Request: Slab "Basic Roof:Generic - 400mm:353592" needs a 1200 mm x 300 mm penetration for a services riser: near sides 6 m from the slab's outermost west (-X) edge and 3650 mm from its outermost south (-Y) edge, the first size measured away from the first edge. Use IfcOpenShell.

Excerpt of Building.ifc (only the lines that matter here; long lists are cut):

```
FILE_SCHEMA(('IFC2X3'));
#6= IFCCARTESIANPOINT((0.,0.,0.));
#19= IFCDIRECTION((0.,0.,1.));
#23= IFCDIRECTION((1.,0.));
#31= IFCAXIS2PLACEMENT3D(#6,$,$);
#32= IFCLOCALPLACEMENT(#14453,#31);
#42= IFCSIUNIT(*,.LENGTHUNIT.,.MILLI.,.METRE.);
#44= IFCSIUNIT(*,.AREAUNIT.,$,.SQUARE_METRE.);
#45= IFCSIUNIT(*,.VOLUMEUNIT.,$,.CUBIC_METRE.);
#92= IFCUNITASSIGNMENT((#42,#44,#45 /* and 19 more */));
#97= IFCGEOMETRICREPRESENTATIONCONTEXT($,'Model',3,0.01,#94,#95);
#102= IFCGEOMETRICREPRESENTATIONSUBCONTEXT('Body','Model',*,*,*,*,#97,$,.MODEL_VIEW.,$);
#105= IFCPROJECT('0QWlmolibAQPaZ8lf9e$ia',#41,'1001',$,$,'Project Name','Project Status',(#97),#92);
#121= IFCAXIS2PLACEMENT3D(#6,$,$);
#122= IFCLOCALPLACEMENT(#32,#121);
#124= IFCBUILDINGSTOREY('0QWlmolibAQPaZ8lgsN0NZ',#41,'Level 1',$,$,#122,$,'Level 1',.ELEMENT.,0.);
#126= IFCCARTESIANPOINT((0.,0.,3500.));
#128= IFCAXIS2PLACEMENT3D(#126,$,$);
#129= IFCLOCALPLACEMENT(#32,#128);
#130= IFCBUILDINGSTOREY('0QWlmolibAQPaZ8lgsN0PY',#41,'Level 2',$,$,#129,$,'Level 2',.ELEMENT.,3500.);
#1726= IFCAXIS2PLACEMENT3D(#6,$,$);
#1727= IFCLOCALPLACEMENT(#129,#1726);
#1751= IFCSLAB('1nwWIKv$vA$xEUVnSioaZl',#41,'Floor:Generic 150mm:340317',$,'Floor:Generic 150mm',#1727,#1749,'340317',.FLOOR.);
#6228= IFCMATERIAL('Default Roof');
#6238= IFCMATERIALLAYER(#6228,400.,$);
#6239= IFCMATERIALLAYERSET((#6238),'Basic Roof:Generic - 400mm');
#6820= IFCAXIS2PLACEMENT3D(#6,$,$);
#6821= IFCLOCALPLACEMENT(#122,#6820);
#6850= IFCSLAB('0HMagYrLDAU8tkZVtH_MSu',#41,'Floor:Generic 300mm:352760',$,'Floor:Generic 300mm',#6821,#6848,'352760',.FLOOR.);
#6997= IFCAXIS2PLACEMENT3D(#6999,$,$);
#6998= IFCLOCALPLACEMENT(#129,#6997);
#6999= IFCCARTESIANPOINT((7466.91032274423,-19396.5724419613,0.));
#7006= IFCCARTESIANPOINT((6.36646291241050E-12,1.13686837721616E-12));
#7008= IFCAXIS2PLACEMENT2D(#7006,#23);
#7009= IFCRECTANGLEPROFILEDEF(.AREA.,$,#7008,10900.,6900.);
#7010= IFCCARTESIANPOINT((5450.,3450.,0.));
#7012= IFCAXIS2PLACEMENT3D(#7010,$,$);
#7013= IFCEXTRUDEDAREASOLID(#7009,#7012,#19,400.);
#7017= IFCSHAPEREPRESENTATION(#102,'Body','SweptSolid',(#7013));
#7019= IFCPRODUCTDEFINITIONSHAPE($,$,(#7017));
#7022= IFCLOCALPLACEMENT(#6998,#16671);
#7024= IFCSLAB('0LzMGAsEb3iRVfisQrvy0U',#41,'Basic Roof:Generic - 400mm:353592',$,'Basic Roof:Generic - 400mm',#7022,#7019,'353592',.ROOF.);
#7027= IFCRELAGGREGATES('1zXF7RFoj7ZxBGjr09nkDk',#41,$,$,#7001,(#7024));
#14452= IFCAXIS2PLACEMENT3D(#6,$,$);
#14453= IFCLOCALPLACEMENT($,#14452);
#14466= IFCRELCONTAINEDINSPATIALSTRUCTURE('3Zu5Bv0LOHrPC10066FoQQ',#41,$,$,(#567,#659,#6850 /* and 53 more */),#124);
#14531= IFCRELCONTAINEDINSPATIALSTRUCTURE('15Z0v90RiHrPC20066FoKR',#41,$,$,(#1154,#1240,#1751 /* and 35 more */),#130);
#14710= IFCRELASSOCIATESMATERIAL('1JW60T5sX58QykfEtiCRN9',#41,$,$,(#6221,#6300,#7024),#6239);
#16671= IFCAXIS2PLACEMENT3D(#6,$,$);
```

```python
import numpy as np
import ifcopenshell
import ifcopenshell.api.feature
import ifcopenshell.api.geometry
import ifcopenshell.api.root
import ifcopenshell.geom
import ifcopenshell.util.placement
import ifcopenshell.util.representation
import ifcopenshell.util.shape
import ifcopenshell.util.unit

model = ifcopenshell.open("Building.ifc")
unit_scale = ifcopenshell.util.unit.calculate_unit_scale(model)
settings = ifcopenshell.geom.settings()


def volume(element):
    """Net volume in cubic metres, openings subtracted."""
    shape = ifcopenshell.geom.create_shape(settings, element)
    return ifcopenshell.util.shape.get_volume(shape.geometry)


slab = model.by_guid("0LzMGAsEb3iRVfisQrvy0U")
before = volume(slab)

# Extent in the slab's own axes, in metres. The edges named are its -X and -Y sides.
slab_shape = ifcopenshell.geom.create_shape(settings, slab)
vertices = ifcopenshell.util.shape.get_vertices(slab_shape.geometry)
x_min, y_min, bottom = vertices.min(axis=0)
top = vertices[:, 2].max()

opening = ifcopenshell.api.root.create_entity(model, ifc_class="IfcOpeningElement", name="Services riser opening")
context = ifcopenshell.util.representation.get_context(model, "Model", "Body", "MODEL_VIEW")
width, depth = 1.2, 0.3
outline = [(0.0, 0.0), (width, 0.0), (width, depth), (0.0, depth), (0.0, 0.0)]
# Overshoot both faces by 50 mm so the cut is clean.
shape = ifcopenshell.api.geometry.add_slab_representation(
    model, context=context, depth=top - bottom + 0.1, polyline=outline
)
ifcopenshell.api.geometry.assign_representation(model, product=opening, representation=shape)

matrix = ifcopenshell.util.placement.get_local_placement(slab.ObjectPlacement)
matrix[:, 3] = matrix @ np.append(np.array([x_min + 6, y_min + 3.65, bottom - 0.05]) / unit_scale, 1.0)
ifcopenshell.api.geometry.edit_object_placement(model, product=opening, matrix=matrix, is_si=False)
ifcopenshell.api.feature.add_feature(model, feature=opening, element=slab)

after = volume(slab)

print(f"slab volume {before:.3f} -> {after:.3f} m3")

model.write("Building_rev.ifc")
```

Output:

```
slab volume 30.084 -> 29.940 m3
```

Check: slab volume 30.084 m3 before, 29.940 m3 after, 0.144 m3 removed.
